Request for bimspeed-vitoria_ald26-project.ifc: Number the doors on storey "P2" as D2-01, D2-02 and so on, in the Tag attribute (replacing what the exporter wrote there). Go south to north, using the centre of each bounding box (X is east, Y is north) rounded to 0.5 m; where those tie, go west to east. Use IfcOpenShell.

First a look at what the model holds.

```python
import ifcopenshell
import ifcopenshell.util.element
import ifcopenshell.util.placement

model = ifcopenshell.open("bimspeed-vitoria_ald26-project.ifc")
print(model.schema)
storey = next(s for s in model.by_type("IfcBuildingStorey") if s.Name == "P2")
doors = [e for e in ifcopenshell.util.element.get_decomposition(storey) if e.is_a("IfcDoor")]
for e in sorted(doors, key=lambda e: e.id()):
    origin = ifcopenshell.util.placement.get_local_placement(e.ObjectPlacement)[:3, 3]
    print(e.id(), e.Tag, e.Name, origin.round(2) + 0.0, sep=" | ")
```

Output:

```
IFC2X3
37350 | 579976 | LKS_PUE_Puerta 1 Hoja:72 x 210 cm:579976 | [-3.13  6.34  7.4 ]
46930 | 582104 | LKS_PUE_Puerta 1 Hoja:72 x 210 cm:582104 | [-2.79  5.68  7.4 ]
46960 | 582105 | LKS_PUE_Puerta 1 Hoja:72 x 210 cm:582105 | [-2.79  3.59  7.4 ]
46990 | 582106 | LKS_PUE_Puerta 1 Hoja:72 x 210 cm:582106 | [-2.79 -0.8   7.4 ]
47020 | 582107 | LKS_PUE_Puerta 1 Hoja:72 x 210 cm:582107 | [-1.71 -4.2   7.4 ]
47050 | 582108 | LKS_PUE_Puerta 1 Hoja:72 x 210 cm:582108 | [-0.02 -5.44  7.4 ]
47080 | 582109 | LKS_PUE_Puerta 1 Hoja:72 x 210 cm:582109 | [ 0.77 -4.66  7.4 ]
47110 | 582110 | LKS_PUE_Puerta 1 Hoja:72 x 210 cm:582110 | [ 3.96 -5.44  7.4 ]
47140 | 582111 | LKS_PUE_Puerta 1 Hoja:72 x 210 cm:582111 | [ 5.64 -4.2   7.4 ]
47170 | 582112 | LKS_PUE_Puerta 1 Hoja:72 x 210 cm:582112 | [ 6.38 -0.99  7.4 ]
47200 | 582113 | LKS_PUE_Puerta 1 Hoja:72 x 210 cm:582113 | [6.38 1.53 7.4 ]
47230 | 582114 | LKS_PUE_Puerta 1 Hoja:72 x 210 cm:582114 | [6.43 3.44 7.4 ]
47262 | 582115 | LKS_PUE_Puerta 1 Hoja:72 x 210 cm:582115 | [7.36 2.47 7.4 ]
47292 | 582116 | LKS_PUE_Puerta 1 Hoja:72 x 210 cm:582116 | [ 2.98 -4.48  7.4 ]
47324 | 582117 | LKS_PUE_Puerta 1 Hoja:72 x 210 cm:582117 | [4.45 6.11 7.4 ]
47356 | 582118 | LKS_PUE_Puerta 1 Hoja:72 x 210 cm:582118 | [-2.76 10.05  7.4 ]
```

```python
import ifcopenshell
import ifcopenshell.geom
import ifcopenshell.util.element
import ifcopenshell.util.shape

model = ifcopenshell.open("bimspeed-vitoria_ald26-project.ifc")
settings = ifcopenshell.geom.settings()
settings.set("use-world-coords", True)


def centre(element):
    shape = ifcopenshell.geom.create_shape(settings, element)
    return ifcopenshell.util.shape.get_bbox_centroid(shape.geometry)


storey = next(s for s in model.by_type("IfcBuildingStorey") if s.Name == "P2")
doors = [e for e in ifcopenshell.util.element.get_decomposition(storey) if e.is_a("IfcDoor")]

# Insertion points can sit at a corner or the storey origin, so sort by the geometry (in metres).
centres = {e: centre(e) for e in doors}
doors.sort(key=lambda e: (round(centres[e][1] / 0.5), centres[e][0]))

for i, e in enumerate(doors, start=1):
    number = f"D2-{i:02d}"
    e.Tag = number
    print(e.id(), number)

model.write("bimspeed-vitoria_ald26-project_updated.ifc")
```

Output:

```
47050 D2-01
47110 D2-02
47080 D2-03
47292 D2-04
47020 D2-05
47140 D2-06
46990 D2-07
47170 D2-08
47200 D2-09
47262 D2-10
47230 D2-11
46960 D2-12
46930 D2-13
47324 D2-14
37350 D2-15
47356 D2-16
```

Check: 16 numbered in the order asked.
